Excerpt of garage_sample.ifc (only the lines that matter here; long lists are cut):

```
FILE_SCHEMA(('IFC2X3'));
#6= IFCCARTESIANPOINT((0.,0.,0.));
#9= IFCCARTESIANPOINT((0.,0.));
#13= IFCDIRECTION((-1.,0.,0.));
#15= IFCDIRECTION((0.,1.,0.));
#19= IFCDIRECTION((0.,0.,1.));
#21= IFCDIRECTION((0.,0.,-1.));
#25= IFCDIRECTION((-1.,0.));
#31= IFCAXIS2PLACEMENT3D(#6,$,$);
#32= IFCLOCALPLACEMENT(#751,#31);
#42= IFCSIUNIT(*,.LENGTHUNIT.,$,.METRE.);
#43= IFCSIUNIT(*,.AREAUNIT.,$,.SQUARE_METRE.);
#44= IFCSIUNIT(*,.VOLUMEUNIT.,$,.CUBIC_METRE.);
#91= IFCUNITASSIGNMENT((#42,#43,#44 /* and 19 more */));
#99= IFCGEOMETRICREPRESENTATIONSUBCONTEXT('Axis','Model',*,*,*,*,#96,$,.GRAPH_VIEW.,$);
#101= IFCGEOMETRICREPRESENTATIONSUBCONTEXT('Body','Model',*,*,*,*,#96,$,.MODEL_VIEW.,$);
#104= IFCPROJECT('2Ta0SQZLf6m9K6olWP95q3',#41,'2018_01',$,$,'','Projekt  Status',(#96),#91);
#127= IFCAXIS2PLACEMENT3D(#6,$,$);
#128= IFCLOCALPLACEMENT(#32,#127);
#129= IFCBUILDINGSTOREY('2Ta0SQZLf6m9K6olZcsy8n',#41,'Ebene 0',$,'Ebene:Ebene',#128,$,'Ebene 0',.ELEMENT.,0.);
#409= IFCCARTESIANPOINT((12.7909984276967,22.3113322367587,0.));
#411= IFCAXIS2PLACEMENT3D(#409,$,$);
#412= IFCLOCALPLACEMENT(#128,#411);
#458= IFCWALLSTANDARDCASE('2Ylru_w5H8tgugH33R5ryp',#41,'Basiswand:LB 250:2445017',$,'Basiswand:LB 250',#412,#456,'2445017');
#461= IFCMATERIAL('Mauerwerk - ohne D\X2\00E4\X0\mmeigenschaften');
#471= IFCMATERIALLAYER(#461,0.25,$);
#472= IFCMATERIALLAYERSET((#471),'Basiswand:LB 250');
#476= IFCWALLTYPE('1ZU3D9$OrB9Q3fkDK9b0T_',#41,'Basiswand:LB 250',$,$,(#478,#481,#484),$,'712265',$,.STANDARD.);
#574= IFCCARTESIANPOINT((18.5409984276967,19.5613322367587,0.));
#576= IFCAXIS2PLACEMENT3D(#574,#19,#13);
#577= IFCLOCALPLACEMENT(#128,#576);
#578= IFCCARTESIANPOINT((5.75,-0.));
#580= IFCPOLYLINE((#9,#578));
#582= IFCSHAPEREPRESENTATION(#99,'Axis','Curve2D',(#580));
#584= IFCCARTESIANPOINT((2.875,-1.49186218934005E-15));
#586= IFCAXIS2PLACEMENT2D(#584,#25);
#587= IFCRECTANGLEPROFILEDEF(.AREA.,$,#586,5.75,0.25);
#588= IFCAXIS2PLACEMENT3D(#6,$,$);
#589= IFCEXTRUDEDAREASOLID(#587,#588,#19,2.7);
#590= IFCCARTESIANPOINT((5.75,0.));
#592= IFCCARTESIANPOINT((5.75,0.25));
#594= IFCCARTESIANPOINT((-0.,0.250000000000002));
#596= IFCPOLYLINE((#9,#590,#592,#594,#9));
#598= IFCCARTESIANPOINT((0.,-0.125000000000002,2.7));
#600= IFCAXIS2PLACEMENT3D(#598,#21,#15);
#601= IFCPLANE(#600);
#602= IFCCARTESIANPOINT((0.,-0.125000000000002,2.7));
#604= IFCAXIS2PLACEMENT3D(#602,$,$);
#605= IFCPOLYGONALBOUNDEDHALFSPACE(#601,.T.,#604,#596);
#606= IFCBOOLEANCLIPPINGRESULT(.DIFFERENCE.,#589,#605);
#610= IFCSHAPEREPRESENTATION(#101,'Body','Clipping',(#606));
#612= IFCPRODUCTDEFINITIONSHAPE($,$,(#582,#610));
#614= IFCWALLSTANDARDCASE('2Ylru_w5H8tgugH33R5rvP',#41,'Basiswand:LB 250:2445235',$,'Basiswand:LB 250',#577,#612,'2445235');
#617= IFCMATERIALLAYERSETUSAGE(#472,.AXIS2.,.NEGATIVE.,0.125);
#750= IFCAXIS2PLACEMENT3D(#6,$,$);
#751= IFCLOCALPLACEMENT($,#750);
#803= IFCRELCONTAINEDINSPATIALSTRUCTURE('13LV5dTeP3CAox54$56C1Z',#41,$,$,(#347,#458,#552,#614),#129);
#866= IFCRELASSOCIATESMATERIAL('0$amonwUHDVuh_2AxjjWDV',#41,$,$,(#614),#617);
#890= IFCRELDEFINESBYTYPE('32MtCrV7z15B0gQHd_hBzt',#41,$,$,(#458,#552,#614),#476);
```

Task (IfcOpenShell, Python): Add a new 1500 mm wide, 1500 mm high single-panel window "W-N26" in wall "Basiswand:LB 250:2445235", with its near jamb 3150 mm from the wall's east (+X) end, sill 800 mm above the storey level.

```python
import numpy as np
import ifcopenshell
import ifcopenshell.api.feature
import ifcopenshell.api.geometry
import ifcopenshell.api.root
import ifcopenshell.api.spatial
import ifcopenshell.api.type
import ifcopenshell.geom
import ifcopenshell.util.element
import ifcopenshell.util.placement
import ifcopenshell.util.representation
import ifcopenshell.util.shape
import ifcopenshell.util.unit

model = ifcopenshell.open("garage_sample.ifc")
unit_scale = ifcopenshell.util.unit.calculate_unit_scale(model)
settings = ifcopenshell.geom.settings()


def volume(element):
    """Net volume in cubic metres, openings subtracted."""
    shape = ifcopenshell.geom.create_shape(settings, element)
    return ifcopenshell.util.shape.get_volume(shape.geometry)


wall = model.by_guid("2Ylru_w5H8tgugH33R5rvP")
storey = ifcopenshell.util.element.get_container(wall, ifc_class="IfcBuildingStorey")
context = ifcopenshell.util.representation.get_context(model, "Model", "Body", "MODEL_VIEW")
before = volume(wall)

width, height, from_end, sill = 1.5, 1.5, 3.15, 0.8  # metres

# The wall runs along its own X axis, and the end named is its -X end.
wall_shape = ifcopenshell.geom.create_shape(settings, wall)
x, y, z = ifcopenshell.util.shape.get_vertices(wall_shape.geometry).T
start = x.min() + from_end
face, thickness = float(y.min()), float(y.max() - y.min())
wall_matrix = ifcopenshell.util.placement.get_local_placement(wall.ObjectPlacement)
level = ifcopenshell.util.placement.get_local_placement(storey.ObjectPlacement)[2, 3]


def in_wall(x, y):
    """Placement at x, y metres in the wall's axes, at sill height."""
    matrix = wall_matrix.copy()
    matrix[:, 3] = wall_matrix @ np.array([x / unit_scale, y / unit_scale, 0.0, 1.0])
    matrix[2, 3] = level + sill / unit_scale
    return matrix


# Opening: a box that overshoots both wall faces by 50 mm.
opening = ifcopenshell.api.root.create_entity(model, ifc_class="IfcOpeningElement")
box = ifcopenshell.api.geometry.add_wall_representation(
    model, context=context, length=width, height=height, thickness=thickness + 0.1
)
ifcopenshell.api.geometry.assign_representation(model, product=opening, representation=box)
ifcopenshell.api.geometry.edit_object_placement(model, product=opening, matrix=in_wall(start, face - 0.05), is_si=False)
ifcopenshell.api.feature.add_feature(model, feature=opening, element=wall)

window = ifcopenshell.api.root.create_entity(model, ifc_class="IfcWindow", name="W-N26")
window.OverallWidth, window.OverallHeight = width / unit_scale, height / unit_scale
body = ifcopenshell.api.geometry.add_window_representation(
    model,
    context=context,
    overall_width=window.OverallWidth,
    overall_height=window.OverallHeight,
    partition_type="SINGLE_PANEL",
)
ifcopenshell.api.geometry.assign_representation(model, product=window, representation=body)
ifcopenshell.api.spatial.assign_container(model, products=[window], relating_structure=storey)
fills = ifcopenshell.api.feature.add_filling(model, opening=opening, element=window)
fills.OwnerHistory = window.OwnerHistory  # required in IFC2X3

# IFC2X3 keeps the operation on the window style.
style = ifcopenshell.api.root.create_entity(model, ifc_class="IfcWindowStyle", name="W-N26")
style.OperationType, style.ConstructionType = "SINGLE_PANEL", "NOTDEFINED"
style.ParameterTakesPrecedence = style.Sizeable = False
ifcopenshell.api.type.assign_type(model, related_objects=[window], relating_type=style)

# Centre the window in the wall's thickness.
ifcopenshell.api.geometry.edit_object_placement(model, product=window, matrix=in_wall(start, face), is_si=False)
window_shape = ifcopenshell.geom.create_shape(settings, window)
depth = ifcopenshell.util.shape.get_vertices(window_shape.geometry)[:, 1]
offset = face + thickness / 2 - (depth.min() + depth.max()) / 2
ifcopenshell.api.geometry.edit_object_placement(model, product=window, matrix=in_wall(start, offset), is_si=False)

after = volume(wall)

print(f"wall volume {before:.3f} -> {after:.3f} m3")

model.write("garage_sample_updated.ifc")
```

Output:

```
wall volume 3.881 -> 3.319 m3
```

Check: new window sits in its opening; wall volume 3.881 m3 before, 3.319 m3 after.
